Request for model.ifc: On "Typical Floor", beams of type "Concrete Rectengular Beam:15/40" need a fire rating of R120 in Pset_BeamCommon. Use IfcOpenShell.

First a look at what the model holds.

```python
import ifcopenshell
import ifcopenshell.util.element

model = ifcopenshell.open("model.ifc")
print(model.schema)
storey = next(s for s in model.by_type("IfcBuildingStorey") if s.Name == "Typical Floor")
beams = [e for e in ifcopenshell.util.element.get_decomposition(storey) if e.is_a("IfcBeam")]
seen = {}
for e in beams:
    element_type = ifcopenshell.util.element.get_type(e)
    key = (element_type.Name if element_type != e and element_type else None, ifcopenshell.util.element.get_pset(e, "Pset_BeamCommon", "FireRating"))
    seen[key] = seen.get(key, 0) + 1
for (name, value), count in sorted(seen.items(), key=str):
    print(count, "x", name, "|", value)
```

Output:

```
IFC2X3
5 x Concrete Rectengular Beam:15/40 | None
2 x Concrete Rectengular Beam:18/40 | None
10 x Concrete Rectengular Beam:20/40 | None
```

```python
import ifcopenshell
import ifcopenshell.api.pset
import ifcopenshell.util.element

model = ifcopenshell.open("model.ifc")

storey = next(s for s in model.by_type("IfcBuildingStorey") if s.Name == "Typical Floor")
beams = [e for e in ifcopenshell.util.element.get_decomposition(storey) if e.is_a("IfcBeam")]

count = 0
for e in beams:
    element_type = ifcopenshell.util.element.get_type(e)
    if element_type in (None, e) or element_type.Name != "Concrete Rectengular Beam:15/40":
        continue
    # add_pset returns the element's existing set when there is one.
    pset = ifcopenshell.api.pset.add_pset(model, product=e, name="Pset_BeamCommon")
    ifcopenshell.api.pset.edit_pset(model, pset=pset, properties={"FireRating": "R120"})
    count += 1

print(count, "beams updated")

model.write("model-out.ifc")
```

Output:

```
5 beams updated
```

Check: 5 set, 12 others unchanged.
